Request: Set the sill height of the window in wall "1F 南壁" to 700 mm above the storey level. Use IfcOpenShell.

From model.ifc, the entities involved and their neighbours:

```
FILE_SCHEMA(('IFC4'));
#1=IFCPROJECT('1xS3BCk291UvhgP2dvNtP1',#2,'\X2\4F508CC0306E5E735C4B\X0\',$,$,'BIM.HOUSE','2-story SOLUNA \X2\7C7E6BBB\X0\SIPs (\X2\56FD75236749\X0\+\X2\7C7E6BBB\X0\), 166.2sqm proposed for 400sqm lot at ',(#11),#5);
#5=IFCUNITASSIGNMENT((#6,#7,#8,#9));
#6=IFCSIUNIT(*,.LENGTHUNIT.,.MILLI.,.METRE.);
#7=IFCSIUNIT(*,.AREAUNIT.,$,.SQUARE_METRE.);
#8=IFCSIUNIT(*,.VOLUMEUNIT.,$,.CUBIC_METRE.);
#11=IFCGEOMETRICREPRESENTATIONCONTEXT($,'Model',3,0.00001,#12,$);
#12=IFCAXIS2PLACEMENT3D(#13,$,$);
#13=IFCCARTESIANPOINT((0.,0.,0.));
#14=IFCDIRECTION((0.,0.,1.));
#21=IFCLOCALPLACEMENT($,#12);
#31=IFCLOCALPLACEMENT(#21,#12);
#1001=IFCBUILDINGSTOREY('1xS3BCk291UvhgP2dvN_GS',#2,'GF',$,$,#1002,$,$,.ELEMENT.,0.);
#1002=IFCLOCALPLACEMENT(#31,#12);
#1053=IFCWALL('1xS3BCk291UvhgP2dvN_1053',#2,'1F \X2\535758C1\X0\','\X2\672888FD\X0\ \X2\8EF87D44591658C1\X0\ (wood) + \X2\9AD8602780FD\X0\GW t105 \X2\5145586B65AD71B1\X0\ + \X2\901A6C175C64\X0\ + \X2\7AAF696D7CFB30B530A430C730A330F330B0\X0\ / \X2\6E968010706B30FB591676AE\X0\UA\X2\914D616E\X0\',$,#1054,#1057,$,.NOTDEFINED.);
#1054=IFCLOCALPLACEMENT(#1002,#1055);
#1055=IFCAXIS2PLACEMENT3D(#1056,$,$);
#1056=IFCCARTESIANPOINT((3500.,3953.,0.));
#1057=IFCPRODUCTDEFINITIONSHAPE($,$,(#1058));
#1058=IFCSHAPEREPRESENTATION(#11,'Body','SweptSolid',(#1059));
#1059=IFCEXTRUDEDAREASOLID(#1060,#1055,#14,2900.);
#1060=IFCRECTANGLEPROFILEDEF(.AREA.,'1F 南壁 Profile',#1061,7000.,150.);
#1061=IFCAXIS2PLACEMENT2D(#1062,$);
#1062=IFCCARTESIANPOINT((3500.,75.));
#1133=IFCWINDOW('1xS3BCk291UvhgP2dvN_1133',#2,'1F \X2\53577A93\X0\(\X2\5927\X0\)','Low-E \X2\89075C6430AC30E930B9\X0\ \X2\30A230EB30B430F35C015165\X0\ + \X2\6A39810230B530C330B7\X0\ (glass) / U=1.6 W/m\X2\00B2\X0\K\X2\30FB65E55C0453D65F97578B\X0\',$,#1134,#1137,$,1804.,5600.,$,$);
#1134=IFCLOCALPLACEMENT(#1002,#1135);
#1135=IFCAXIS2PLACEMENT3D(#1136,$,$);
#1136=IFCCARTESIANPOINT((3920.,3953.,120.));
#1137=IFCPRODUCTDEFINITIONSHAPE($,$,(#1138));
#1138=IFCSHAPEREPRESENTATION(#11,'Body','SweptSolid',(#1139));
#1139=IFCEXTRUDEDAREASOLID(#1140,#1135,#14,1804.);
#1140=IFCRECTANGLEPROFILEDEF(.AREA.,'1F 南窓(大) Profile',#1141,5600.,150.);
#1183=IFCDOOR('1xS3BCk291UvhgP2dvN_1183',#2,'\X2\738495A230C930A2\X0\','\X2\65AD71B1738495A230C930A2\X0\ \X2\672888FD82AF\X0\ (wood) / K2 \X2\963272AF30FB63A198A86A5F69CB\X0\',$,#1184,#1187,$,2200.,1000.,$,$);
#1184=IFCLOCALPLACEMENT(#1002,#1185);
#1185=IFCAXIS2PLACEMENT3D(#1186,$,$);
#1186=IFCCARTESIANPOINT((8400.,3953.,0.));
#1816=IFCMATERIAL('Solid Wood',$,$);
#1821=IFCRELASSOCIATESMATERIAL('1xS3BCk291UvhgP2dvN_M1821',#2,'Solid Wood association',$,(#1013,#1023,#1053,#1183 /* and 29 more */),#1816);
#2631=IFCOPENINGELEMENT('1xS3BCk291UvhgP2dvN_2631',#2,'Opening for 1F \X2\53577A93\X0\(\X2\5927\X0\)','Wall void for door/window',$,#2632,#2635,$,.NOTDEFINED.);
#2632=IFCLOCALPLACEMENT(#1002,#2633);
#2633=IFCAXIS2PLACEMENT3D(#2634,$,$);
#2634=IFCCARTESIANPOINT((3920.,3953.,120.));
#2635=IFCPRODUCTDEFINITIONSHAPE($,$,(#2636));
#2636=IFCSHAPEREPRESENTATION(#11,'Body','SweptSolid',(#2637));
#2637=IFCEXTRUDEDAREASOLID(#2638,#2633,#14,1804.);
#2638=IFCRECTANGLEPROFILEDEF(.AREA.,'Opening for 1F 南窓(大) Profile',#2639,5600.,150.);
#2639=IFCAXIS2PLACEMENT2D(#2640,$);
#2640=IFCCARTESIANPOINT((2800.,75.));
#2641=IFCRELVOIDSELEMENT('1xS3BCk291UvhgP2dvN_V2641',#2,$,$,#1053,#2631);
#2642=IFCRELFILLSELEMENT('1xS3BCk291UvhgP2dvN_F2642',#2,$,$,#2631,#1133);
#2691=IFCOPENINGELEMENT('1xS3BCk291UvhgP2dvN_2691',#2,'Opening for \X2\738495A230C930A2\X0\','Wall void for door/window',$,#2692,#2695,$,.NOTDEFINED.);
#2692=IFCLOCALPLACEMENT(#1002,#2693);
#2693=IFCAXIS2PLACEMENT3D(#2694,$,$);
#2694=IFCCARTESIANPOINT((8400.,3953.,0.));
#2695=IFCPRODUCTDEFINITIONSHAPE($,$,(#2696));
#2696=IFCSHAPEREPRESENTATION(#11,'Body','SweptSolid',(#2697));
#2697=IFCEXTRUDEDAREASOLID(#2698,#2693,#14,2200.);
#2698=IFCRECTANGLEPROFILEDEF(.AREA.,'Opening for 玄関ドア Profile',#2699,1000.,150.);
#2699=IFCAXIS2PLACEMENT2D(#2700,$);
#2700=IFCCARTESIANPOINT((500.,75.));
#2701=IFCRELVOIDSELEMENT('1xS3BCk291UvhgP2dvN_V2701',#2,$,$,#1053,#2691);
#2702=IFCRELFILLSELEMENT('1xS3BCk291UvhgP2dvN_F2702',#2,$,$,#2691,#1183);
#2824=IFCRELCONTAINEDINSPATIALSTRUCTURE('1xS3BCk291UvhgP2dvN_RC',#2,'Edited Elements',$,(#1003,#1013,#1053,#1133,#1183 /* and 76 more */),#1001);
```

```python
import numpy as np
import ifcopenshell
import ifcopenshell.api.geometry
import ifcopenshell.geom
import ifcopenshell.util.element
import ifcopenshell.util.placement
import ifcopenshell.util.shape
import ifcopenshell.util.unit

model = ifcopenshell.open("model.ifc")
unit_scale = ifcopenshell.util.unit.calculate_unit_scale(model)

window = model.by_id(1133)
opening = window.FillsVoids[0].RelatingOpeningElement
storey = ifcopenshell.util.element.get_container(window, ifc_class="IfcBuildingStorey")
level = ifcopenshell.util.placement.get_local_placement(storey.ObjectPlacement)[2, 3]

# The opening's origin need not be at the sill, so measure its lowest point.
shape = ifcopenshell.geom.create_shape(ifcopenshell.geom.settings(), opening)
bottom = ifcopenshell.util.shape.get_shape_bottom_elevation(shape, shape.geometry) / unit_scale
dz = level + 700.0 - bottom

shift = np.array([0.0, 0.0, dz])
# The window is not placed relative to its opening, so move both.
for product in (opening, window):
    matrix = ifcopenshell.util.placement.get_local_placement(product.ObjectPlacement)
    matrix[:3, 3] += shift
    ifcopenshell.api.geometry.edit_object_placement(model, product=product, matrix=matrix, is_si=False)

print(f"moved by {dz * unit_scale:+.3f} m")

model.write("model_edited.ifc")
```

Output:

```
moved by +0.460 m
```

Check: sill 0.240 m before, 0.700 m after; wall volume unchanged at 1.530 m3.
